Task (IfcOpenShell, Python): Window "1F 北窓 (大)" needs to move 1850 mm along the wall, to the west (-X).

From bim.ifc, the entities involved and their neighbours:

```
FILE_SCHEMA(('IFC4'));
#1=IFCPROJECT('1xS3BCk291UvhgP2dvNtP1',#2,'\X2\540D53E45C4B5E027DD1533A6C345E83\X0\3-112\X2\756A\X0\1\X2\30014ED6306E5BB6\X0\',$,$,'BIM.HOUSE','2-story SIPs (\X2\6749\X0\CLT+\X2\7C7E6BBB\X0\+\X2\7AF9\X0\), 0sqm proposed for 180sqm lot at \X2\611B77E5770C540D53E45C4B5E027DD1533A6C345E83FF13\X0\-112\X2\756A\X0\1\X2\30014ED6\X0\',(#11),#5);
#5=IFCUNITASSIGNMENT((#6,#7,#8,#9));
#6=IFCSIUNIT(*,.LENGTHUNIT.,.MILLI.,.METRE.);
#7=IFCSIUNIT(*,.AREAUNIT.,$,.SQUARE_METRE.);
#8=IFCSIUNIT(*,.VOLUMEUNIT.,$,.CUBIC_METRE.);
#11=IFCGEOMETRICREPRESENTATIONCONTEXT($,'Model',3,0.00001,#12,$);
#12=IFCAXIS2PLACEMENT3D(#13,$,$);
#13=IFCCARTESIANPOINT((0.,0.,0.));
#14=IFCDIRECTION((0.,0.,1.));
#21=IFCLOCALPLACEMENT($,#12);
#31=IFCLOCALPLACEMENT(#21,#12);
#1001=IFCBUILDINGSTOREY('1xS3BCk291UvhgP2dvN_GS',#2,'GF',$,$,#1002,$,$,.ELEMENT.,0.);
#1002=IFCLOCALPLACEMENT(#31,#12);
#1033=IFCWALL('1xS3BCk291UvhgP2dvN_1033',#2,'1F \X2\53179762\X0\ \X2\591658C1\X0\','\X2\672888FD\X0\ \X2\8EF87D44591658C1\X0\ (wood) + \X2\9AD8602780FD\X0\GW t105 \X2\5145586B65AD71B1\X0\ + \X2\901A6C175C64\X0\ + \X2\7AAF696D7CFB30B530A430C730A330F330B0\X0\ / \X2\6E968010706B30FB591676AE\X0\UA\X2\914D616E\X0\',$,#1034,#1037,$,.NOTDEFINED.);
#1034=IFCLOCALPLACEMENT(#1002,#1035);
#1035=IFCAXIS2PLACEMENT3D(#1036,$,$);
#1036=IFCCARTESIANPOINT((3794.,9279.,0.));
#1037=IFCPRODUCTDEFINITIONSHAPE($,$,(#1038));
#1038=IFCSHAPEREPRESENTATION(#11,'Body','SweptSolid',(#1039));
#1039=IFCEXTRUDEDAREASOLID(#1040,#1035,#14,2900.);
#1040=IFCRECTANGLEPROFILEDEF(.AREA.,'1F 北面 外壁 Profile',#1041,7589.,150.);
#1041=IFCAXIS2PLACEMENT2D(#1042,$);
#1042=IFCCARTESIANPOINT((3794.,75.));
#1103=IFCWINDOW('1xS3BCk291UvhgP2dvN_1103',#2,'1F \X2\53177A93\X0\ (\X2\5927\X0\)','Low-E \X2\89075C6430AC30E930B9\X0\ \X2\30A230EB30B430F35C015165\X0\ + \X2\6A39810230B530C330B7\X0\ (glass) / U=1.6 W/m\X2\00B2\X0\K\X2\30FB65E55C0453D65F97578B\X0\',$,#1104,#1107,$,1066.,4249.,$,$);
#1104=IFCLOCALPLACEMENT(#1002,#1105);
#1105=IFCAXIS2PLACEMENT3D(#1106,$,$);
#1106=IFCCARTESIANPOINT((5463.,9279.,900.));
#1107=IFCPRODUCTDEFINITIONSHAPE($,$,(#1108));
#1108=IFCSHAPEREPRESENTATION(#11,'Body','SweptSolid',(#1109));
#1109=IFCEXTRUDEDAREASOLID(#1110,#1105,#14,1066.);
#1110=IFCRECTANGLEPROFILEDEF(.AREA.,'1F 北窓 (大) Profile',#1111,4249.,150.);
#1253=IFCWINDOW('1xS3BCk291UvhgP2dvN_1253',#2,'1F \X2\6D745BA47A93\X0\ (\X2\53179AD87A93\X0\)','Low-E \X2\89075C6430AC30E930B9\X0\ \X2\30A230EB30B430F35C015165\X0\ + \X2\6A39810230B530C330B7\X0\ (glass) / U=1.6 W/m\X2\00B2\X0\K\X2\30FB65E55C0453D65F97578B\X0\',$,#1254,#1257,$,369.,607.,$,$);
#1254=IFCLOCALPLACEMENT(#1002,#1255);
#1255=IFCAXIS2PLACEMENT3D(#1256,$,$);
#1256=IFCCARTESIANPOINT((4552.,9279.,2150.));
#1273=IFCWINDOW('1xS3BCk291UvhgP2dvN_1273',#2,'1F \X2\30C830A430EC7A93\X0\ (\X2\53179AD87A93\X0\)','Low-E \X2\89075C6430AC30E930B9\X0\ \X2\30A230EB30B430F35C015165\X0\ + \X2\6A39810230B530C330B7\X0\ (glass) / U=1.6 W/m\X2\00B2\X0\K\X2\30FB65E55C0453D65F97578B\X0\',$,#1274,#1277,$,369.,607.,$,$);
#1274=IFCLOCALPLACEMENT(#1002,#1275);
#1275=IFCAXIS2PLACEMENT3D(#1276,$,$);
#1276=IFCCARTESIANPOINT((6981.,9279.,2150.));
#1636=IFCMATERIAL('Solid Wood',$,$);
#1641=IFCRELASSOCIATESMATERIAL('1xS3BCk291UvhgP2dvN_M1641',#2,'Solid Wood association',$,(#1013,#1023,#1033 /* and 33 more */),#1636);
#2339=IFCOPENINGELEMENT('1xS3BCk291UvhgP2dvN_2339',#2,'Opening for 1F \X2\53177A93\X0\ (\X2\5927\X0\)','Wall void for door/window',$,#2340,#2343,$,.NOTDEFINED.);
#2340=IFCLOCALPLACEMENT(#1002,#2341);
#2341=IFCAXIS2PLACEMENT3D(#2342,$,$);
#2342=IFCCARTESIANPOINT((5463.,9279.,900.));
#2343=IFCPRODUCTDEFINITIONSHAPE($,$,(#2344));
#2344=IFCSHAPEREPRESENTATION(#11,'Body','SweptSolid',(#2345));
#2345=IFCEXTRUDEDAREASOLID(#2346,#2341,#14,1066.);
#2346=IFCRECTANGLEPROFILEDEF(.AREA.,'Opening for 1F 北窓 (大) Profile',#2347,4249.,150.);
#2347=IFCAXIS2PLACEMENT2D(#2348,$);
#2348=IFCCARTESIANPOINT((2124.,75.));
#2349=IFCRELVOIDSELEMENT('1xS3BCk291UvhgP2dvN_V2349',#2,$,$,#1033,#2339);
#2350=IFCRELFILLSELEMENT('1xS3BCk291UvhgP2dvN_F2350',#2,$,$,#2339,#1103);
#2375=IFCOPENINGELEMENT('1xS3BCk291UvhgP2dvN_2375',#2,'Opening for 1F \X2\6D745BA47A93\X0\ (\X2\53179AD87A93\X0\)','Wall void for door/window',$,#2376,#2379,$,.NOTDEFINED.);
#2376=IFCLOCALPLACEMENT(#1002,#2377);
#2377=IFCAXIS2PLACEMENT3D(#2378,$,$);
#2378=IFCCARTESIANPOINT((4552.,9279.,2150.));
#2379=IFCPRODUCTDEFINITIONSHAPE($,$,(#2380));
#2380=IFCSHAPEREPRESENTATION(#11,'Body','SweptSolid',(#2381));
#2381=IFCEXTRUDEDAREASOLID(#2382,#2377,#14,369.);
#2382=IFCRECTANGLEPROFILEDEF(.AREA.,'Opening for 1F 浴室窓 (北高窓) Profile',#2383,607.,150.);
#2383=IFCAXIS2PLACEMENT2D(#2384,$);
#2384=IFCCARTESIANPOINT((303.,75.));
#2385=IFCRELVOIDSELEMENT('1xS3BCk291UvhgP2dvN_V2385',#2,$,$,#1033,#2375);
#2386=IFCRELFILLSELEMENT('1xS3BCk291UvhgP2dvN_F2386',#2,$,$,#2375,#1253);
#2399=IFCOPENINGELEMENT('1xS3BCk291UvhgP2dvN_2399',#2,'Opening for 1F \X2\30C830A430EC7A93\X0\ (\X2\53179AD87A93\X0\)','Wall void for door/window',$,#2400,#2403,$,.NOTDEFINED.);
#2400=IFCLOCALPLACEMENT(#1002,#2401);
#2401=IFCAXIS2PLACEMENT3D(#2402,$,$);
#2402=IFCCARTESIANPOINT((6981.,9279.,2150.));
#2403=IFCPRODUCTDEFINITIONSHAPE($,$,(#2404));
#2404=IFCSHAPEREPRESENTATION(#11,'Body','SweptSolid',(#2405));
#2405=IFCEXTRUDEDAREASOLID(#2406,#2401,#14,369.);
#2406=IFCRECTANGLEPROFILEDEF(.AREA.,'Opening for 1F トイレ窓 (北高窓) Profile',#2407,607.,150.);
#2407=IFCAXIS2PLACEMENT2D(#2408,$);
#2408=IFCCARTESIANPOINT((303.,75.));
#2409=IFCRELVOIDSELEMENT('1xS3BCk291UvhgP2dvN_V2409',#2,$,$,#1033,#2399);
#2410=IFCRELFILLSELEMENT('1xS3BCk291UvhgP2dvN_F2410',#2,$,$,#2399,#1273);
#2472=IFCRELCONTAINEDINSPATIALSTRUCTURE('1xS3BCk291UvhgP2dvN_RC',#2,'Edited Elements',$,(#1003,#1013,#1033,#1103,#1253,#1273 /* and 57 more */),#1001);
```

```python
import ifcopenshell
import ifcopenshell.api.geometry
import ifcopenshell.util.placement
import ifcopenshell.util.unit

model = ifcopenshell.open("bim.ifc")
unit_scale = ifcopenshell.util.unit.calculate_unit_scale(model)

window = model.by_guid("1xS3BCk291UvhgP2dvN_1103")
opening = window.FillsVoids[0].RelatingOpeningElement
wall = opening.VoidsElements[0].RelatingBuildingElement

wall_matrix = ifcopenshell.util.placement.get_local_placement(wall.ObjectPlacement)
shift = wall_matrix[:3, 0] * -1.85 / unit_scale
before = ifcopenshell.util.placement.get_local_placement(window.ObjectPlacement)[:3, 3].copy()

# The window is not placed relative to its opening, so move both.
for product in (opening, window):
    matrix = ifcopenshell.util.placement.get_local_placement(product.ObjectPlacement)
    matrix[:3, 3] += shift
    ifcopenshell.api.geometry.edit_object_placement(model, product=product, matrix=matrix, is_si=False)

after = ifcopenshell.util.placement.get_local_placement(window.ObjectPlacement)[:3, 3]
print("window moved by", (after - before).round(3) + 0.0)

model.write("bim_v2.ifc")
```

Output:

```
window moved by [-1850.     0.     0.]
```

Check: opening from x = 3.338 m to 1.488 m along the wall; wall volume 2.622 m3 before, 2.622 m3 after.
